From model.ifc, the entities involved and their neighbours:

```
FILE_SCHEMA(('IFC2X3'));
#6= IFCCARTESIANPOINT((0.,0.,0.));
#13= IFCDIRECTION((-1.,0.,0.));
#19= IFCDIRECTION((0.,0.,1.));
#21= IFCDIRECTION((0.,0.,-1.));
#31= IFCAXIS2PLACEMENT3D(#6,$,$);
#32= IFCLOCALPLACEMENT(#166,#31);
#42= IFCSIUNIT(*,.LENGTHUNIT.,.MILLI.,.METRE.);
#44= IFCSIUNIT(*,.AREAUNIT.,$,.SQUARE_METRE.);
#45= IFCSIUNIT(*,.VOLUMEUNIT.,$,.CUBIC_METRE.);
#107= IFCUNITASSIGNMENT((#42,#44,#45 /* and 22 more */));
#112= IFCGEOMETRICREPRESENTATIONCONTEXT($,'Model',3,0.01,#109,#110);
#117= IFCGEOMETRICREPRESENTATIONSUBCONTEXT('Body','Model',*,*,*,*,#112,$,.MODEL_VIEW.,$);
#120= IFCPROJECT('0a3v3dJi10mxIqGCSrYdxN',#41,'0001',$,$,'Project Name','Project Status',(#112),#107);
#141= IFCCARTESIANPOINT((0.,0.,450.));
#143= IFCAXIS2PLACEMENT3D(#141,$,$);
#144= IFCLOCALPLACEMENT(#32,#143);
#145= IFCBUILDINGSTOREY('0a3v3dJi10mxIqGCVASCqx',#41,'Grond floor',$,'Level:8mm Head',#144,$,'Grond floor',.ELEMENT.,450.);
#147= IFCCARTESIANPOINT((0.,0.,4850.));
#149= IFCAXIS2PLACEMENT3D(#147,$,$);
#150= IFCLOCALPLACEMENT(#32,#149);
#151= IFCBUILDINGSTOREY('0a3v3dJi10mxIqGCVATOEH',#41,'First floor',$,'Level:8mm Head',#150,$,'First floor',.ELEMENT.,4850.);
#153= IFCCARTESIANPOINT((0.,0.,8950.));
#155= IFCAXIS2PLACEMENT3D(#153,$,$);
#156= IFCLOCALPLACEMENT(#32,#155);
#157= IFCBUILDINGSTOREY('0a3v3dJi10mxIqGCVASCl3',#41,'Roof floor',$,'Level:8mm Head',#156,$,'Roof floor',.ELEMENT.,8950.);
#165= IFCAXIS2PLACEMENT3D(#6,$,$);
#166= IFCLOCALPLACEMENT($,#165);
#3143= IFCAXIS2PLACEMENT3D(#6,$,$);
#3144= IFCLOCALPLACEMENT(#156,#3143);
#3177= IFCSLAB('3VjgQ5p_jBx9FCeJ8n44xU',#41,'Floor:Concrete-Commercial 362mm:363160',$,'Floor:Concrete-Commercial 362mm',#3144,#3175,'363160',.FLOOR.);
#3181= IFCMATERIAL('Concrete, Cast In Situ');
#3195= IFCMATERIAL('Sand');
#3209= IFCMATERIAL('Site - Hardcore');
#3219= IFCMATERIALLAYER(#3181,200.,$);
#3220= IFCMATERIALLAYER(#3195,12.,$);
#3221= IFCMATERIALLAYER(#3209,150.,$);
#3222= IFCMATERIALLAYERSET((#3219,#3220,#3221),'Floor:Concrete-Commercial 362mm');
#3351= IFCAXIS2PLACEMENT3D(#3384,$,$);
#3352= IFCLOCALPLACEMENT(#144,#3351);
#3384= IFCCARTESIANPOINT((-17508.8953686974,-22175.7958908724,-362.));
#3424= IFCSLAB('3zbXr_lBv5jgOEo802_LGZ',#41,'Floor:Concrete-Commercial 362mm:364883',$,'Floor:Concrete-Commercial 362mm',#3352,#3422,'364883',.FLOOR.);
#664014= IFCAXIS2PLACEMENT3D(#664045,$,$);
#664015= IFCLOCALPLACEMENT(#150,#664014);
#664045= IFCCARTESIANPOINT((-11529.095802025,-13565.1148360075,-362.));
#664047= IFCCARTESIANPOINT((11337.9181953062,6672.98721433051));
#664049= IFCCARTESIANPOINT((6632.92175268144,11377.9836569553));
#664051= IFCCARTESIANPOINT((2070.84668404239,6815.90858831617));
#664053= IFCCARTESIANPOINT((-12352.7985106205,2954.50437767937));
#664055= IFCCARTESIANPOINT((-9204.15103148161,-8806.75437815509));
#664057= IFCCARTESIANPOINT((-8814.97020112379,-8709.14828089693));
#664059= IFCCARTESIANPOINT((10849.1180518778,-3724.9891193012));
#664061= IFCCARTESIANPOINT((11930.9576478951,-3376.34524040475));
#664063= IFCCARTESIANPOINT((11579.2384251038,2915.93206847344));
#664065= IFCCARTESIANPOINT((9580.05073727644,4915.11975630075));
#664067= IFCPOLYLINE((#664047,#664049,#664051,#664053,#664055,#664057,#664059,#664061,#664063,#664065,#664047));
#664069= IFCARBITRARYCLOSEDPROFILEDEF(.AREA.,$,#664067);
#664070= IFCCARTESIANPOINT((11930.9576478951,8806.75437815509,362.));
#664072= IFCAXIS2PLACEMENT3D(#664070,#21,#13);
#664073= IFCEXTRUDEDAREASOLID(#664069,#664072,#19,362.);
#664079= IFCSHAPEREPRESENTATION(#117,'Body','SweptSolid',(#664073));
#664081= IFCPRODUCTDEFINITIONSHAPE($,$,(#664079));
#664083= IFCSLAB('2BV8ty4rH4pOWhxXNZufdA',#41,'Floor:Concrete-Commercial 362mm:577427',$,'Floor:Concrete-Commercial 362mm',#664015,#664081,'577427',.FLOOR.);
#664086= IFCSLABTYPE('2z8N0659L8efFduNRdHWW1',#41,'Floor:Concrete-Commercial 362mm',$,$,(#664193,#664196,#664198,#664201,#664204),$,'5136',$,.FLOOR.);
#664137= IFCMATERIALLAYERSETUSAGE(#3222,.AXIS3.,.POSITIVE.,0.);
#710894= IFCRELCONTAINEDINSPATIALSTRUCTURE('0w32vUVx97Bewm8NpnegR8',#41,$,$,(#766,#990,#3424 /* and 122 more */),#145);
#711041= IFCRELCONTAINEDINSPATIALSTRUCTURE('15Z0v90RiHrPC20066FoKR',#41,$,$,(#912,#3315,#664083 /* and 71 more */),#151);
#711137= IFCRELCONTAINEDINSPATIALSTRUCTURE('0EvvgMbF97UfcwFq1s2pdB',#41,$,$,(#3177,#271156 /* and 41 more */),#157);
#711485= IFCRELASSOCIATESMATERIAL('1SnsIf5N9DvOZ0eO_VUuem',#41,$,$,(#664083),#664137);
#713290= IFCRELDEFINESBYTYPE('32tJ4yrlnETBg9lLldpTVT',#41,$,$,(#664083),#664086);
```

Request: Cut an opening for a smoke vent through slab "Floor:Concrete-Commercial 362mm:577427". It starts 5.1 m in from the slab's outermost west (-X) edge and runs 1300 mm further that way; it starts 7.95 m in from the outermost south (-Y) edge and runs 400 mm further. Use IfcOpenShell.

```python
import numpy as np
import ifcopenshell
import ifcopenshell.api.feature
import ifcopenshell.api.geometry
import ifcopenshell.api.root
import ifcopenshell.geom
import ifcopenshell.util.placement
import ifcopenshell.util.representation
import ifcopenshell.util.shape
import ifcopenshell.util.unit

model = ifcopenshell.open("model.ifc")
unit_scale = ifcopenshell.util.unit.calculate_unit_scale(model)
settings = ifcopenshell.geom.settings()


def volume(element):
    """Net volume in cubic metres, openings subtracted."""
    shape = ifcopenshell.geom.create_shape(settings, element)
    return ifcopenshell.util.shape.get_volume(shape.geometry)


slab = model.by_guid("2BV8ty4rH4pOWhxXNZufdA")
before = volume(slab)

# Extent in the slab's own axes, in metres. The edges named are its -X and -Y sides.
slab_shape = ifcopenshell.geom.create_shape(settings, slab)
vertices = ifcopenshell.util.shape.get_vertices(slab_shape.geometry)
x_min, y_min, bottom = vertices.min(axis=0)
top = vertices[:, 2].max()

opening = ifcopenshell.api.root.create_entity(model, ifc_class="IfcOpeningElement", name="Smoke vent opening")
context = ifcopenshell.util.representation.get_context(model, "Model", "Body", "MODEL_VIEW")
width, depth = 1.3, 0.4
outline = [(0.0, 0.0), (width, 0.0), (width, depth), (0.0, depth), (0.0, 0.0)]
# Overshoot both faces by 50 mm so the cut is clean.
shape = ifcopenshell.api.geometry.add_slab_representation(
    model, context=context, depth=top - bottom + 0.1, polyline=outline
)
ifcopenshell.api.geometry.assign_representation(model, product=opening, representation=shape)

matrix = ifcopenshell.util.placement.get_local_placement(slab.ObjectPlacement)
matrix[:, 3] = matrix @ np.append(np.array([x_min + 5.1, y_min + 7.95, bottom - 0.05]) / unit_scale, 1.0)
ifcopenshell.api.geometry.edit_object_placement(model, product=opening, matrix=matrix, is_si=False)
ifcopenshell.api.feature.add_feature(model, feature=opening, element=slab)

after = volume(slab)

print(f"slab volume {before:.3f} -> {after:.3f} m3")

model.write("model_updated.ifc")
```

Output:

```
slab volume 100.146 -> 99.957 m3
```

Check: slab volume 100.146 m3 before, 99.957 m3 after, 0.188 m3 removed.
